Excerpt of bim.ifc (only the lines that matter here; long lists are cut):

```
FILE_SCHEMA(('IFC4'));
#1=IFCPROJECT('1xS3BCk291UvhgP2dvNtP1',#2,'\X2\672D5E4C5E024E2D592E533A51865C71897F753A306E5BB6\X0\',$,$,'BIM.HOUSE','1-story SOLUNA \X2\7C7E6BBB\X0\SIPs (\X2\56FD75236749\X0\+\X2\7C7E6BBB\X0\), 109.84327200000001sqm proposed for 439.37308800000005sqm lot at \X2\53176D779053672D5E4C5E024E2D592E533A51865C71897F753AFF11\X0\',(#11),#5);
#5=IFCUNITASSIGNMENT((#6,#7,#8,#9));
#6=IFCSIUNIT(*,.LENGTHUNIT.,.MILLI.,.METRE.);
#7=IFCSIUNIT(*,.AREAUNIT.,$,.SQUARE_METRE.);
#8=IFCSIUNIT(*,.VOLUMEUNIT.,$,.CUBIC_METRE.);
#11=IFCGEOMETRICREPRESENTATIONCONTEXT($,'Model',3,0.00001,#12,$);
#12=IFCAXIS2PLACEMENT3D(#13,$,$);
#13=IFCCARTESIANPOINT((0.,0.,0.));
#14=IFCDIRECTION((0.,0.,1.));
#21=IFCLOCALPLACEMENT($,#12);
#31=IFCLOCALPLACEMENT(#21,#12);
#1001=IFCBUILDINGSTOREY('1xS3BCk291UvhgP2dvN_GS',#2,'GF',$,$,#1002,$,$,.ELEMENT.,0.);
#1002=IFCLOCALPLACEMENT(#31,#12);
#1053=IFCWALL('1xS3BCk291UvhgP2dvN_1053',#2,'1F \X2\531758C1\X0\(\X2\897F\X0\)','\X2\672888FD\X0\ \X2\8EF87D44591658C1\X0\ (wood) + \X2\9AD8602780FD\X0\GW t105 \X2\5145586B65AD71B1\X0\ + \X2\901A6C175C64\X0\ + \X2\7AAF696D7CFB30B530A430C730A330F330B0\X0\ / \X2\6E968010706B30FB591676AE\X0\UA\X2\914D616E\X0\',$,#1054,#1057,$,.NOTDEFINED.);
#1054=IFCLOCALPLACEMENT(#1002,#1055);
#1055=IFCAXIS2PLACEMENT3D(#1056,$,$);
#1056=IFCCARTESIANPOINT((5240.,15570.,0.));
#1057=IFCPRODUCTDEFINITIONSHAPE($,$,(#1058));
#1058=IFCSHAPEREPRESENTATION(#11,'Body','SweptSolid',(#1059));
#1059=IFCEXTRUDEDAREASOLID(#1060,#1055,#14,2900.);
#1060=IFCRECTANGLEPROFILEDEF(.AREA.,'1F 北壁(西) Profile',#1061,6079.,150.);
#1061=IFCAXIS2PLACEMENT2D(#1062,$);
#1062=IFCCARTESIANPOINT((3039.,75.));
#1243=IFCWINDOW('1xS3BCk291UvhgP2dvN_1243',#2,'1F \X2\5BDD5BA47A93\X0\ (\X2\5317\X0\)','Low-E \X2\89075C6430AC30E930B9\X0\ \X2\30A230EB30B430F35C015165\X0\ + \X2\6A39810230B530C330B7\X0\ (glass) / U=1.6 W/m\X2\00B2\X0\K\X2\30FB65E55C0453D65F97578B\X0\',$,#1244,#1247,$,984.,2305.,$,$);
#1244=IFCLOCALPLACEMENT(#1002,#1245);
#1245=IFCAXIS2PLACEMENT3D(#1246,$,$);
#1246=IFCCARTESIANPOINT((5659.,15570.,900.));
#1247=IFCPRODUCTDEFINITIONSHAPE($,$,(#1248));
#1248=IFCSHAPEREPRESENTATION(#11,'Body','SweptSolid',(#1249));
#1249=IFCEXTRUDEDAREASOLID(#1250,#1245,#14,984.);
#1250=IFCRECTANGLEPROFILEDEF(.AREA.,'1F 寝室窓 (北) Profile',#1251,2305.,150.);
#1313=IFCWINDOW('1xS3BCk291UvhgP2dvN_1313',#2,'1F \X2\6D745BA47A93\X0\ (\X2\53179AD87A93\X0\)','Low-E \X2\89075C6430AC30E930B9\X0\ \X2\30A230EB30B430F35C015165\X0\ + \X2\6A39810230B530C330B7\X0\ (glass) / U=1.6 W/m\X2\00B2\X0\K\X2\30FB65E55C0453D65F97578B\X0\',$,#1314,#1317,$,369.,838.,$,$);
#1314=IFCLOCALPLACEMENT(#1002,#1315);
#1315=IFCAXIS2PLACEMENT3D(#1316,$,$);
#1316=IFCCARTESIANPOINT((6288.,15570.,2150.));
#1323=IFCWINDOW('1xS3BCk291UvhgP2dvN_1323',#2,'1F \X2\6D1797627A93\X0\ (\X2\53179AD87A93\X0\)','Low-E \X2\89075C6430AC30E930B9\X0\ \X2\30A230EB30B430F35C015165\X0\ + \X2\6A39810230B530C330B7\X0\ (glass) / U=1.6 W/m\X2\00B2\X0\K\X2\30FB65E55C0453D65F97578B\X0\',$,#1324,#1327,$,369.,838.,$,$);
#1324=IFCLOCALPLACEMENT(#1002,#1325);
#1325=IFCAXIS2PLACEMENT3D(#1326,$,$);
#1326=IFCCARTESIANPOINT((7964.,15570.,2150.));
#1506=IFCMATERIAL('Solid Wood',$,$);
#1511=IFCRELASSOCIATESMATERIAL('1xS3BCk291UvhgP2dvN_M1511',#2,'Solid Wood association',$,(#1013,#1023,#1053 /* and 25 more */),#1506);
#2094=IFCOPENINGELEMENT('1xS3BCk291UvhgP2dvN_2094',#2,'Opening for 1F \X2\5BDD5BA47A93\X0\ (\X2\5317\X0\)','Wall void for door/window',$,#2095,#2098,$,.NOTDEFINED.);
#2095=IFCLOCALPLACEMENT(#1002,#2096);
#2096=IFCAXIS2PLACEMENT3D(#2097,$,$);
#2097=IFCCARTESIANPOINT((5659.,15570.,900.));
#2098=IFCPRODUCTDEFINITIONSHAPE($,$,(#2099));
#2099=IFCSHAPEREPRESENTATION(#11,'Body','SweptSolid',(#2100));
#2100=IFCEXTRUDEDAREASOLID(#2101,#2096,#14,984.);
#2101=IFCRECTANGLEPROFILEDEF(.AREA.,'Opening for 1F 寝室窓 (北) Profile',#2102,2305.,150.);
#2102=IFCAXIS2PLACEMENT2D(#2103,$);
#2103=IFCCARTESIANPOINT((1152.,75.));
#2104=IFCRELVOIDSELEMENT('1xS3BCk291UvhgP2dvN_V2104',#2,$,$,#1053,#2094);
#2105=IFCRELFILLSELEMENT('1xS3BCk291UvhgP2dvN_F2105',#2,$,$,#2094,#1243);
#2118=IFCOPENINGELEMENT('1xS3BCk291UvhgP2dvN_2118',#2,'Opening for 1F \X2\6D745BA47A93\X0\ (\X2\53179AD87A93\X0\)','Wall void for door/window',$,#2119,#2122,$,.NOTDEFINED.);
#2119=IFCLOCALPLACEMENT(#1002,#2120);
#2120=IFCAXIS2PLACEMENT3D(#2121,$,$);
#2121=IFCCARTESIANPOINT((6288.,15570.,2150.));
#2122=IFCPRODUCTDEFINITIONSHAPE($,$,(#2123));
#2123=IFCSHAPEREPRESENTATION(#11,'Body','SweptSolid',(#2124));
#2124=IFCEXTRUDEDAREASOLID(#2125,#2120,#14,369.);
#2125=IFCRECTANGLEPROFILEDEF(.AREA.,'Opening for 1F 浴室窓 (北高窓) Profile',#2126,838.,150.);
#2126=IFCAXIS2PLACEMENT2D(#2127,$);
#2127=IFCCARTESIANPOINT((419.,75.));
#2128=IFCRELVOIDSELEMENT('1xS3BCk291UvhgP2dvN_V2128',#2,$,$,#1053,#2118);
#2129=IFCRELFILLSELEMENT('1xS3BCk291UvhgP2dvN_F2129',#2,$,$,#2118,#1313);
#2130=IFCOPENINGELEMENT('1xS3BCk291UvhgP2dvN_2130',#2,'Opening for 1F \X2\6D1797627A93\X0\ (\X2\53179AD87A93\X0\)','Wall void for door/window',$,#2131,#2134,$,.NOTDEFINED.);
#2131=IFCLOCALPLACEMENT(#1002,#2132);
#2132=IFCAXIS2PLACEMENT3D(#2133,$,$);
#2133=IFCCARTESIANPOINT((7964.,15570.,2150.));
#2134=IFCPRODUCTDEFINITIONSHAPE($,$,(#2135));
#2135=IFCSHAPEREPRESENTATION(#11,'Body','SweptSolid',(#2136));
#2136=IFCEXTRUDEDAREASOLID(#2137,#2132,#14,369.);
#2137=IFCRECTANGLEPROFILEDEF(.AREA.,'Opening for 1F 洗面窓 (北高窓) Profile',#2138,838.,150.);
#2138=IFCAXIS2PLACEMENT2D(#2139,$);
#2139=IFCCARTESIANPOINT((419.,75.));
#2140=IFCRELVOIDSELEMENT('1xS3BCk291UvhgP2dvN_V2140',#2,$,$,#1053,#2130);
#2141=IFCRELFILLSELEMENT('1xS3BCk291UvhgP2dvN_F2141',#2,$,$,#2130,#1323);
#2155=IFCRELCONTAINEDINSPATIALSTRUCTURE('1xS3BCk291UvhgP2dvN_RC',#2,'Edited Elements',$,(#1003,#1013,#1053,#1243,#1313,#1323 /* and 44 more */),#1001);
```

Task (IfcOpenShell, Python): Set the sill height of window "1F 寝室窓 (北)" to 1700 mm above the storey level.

```python
import numpy as np
import ifcopenshell
import ifcopenshell.api.geometry
import ifcopenshell.geom
import ifcopenshell.util.element
import ifcopenshell.util.placement
import ifcopenshell.util.shape
import ifcopenshell.util.unit

model = ifcopenshell.open("bim.ifc")
unit_scale = ifcopenshell.util.unit.calculate_unit_scale(model)

window = model.by_guid("1xS3BCk291UvhgP2dvN_1243")
opening = window.FillsVoids[0].RelatingOpeningElement
storey = ifcopenshell.util.element.get_container(window, ifc_class="IfcBuildingStorey")
level = ifcopenshell.util.placement.get_local_placement(storey.ObjectPlacement)[2, 3]

# The opening's origin need not be at the sill, so measure its lowest point.
shape = ifcopenshell.geom.create_shape(ifcopenshell.geom.settings(), opening)
bottom = ifcopenshell.util.shape.get_shape_bottom_elevation(shape, shape.geometry) / unit_scale
dz = level + 1700.0 - bottom

shift = np.array([0.0, 0.0, dz])
# The window is not placed relative to its opening, so move both.
for product in (opening, window):
    matrix = ifcopenshell.util.placement.get_local_placement(product.ObjectPlacement)
    matrix[:3, 3] += shift
    ifcopenshell.api.geometry.edit_object_placement(model, product=product, matrix=matrix, is_si=False)

print(f"moved by {dz * unit_scale:+.3f} m")

model.write("bim_edited.ifc")
```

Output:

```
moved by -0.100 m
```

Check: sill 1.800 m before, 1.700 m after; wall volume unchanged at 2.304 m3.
